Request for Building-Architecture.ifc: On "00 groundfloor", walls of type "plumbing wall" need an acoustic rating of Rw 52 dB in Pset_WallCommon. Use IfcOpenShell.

First a look at what the model holds.

```python
import ifcopenshell
import ifcopenshell.util.element

model = ifcopenshell.open("Building-Architecture.ifc")
print(model.schema)
storey = next(s for s in model.by_type("IfcBuildingStorey") if s.Name == "00 groundfloor")
walls = [e for e in ifcopenshell.util.element.get_decomposition(storey) if e.is_a("IfcWall")]
seen = {}
for e in walls:
    element_type = ifcopenshell.util.element.get_type(e)
    key = (element_type.Name if element_type != e and element_type else None, ifcopenshell.util.element.get_pset(e, "Pset_WallCommon", "AcousticRating"))
    seen[key] = seen.get(key, 0) + 1
for (name, value), count in sorted(seen.items(), key=str):
    print(count, "x", name, "|", value)
```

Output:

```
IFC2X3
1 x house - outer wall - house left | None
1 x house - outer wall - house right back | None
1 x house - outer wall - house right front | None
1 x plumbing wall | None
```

```python
import ifcopenshell
import ifcopenshell.api.pset
import ifcopenshell.util.element

model = ifcopenshell.open("Building-Architecture.ifc")

storey = next(s for s in model.by_type("IfcBuildingStorey") if s.Name == "00 groundfloor")
walls = [e for e in ifcopenshell.util.element.get_decomposition(storey) if e.is_a("IfcWall")]

count = 0
for e in walls:
    element_type = ifcopenshell.util.element.get_type(e)
    if element_type in (None, e) or element_type.Name != "plumbing wall":
        continue
    # add_pset returns the element's existing set when there is one.
    pset = ifcopenshell.api.pset.add_pset(model, product=e, name="Pset_WallCommon")
    ifcopenshell.api.pset.edit_pset(model, pset=pset, properties={"AcousticRating": "Rw 52 dB"})
    count += 1

print(count, "walls updated")

model.write("Building-Architecture_rev.ifc")
```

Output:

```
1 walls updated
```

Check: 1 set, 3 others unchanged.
